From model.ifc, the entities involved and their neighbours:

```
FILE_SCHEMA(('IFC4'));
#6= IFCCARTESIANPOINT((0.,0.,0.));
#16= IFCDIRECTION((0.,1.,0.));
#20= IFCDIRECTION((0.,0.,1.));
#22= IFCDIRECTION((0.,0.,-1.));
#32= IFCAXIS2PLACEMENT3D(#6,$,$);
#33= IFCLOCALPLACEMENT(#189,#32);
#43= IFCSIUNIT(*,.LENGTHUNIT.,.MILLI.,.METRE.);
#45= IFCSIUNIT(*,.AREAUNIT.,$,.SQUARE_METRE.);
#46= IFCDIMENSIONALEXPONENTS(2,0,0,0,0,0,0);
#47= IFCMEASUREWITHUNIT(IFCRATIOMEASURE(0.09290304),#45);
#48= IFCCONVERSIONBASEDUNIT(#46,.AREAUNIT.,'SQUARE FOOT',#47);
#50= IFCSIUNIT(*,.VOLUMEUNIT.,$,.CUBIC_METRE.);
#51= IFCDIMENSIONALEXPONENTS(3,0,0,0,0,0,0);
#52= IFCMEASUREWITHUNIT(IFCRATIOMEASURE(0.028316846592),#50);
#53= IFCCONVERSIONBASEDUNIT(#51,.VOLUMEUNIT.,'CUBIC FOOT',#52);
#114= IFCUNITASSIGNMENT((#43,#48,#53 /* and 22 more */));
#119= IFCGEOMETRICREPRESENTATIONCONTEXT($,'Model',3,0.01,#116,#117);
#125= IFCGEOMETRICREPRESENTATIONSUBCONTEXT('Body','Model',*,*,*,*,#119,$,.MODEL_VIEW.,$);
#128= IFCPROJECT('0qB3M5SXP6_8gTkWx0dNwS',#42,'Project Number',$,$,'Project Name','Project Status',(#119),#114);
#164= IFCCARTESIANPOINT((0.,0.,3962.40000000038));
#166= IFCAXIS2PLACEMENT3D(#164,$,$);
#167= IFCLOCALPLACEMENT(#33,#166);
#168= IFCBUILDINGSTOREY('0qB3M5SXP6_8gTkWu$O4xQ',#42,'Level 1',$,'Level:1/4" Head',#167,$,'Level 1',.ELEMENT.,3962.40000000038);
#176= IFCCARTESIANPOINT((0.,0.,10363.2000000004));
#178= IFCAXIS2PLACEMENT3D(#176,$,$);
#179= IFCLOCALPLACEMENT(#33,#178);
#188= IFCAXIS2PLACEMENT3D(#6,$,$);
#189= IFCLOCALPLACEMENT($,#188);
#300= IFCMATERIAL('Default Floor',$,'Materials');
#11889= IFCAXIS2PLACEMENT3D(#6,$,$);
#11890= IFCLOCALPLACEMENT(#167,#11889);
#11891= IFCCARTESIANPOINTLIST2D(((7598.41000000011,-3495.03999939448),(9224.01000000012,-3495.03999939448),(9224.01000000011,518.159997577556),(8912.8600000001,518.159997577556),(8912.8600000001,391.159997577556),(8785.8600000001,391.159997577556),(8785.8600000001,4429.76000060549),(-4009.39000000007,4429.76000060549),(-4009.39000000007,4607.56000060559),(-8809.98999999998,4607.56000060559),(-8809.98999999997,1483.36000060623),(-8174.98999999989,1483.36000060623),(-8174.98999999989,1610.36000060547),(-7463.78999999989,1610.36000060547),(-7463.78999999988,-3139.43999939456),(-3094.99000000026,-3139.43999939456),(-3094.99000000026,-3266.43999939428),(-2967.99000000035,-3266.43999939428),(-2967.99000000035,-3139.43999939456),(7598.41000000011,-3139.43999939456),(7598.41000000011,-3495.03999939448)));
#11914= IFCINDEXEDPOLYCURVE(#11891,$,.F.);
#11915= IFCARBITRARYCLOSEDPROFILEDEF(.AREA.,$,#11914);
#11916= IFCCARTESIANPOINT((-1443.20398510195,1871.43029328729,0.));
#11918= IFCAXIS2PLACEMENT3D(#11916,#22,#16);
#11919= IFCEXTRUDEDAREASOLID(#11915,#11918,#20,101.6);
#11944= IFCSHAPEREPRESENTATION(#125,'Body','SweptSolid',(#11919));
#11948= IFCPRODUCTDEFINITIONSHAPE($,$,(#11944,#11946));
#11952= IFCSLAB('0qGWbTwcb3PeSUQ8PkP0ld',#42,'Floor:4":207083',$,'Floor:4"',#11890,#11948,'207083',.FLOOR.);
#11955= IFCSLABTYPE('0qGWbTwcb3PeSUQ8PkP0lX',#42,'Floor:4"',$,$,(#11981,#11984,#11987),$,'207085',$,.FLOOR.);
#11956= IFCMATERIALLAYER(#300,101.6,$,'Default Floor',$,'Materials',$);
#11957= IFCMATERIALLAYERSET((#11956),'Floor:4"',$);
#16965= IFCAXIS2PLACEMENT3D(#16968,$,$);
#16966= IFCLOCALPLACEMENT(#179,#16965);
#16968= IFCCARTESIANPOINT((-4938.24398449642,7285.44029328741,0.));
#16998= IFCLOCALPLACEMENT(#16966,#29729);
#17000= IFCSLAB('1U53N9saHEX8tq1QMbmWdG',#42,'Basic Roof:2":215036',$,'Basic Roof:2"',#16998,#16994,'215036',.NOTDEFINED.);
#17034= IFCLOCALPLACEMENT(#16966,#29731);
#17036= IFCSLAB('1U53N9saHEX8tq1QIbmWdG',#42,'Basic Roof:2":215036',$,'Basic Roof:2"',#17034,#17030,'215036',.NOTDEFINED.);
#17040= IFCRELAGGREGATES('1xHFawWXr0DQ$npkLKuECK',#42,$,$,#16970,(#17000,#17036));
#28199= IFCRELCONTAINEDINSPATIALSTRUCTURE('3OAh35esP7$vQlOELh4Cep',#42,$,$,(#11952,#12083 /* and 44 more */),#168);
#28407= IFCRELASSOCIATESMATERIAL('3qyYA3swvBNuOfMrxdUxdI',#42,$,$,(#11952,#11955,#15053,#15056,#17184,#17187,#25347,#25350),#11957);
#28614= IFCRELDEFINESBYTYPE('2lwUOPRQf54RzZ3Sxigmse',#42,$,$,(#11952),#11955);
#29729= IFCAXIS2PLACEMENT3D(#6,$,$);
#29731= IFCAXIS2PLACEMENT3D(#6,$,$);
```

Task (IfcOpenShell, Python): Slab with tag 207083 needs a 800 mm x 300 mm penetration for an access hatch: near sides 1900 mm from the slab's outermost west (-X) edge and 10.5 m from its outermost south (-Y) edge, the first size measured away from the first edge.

```python
import numpy as np
import ifcopenshell
import ifcopenshell.api.feature
import ifcopenshell.api.geometry
import ifcopenshell.api.root
import ifcopenshell.geom
import ifcopenshell.util.placement
import ifcopenshell.util.representation
import ifcopenshell.util.shape
import ifcopenshell.util.unit

model = ifcopenshell.open("model.ifc")
unit_scale = ifcopenshell.util.unit.calculate_unit_scale(model)
settings = ifcopenshell.geom.settings()


def volume(element):
    """Net volume in cubic metres, openings subtracted."""
    shape = ifcopenshell.geom.create_shape(settings, element)
    return ifcopenshell.util.shape.get_volume(shape.geometry)


slab = model.by_guid("0qGWbTwcb3PeSUQ8PkP0ld")
before = volume(slab)

# Extent in the slab's own axes, in metres. The edges named are its -X and -Y sides.
slab_shape = ifcopenshell.geom.create_shape(settings, slab)
vertices = ifcopenshell.util.shape.get_vertices(slab_shape.geometry)
x_min, y_min, bottom = vertices.min(axis=0)
top = vertices[:, 2].max()

opening = ifcopenshell.api.root.create_entity(model, ifc_class="IfcOpeningElement", name="Access hatch opening", predefined_type="OPENING")
context = ifcopenshell.util.representation.get_context(model, "Model", "Body", "MODEL_VIEW")
width, depth = 0.8, 0.3
outline = [(0.0, 0.0), (width, 0.0), (width, depth), (0.0, depth), (0.0, 0.0)]
# Overshoot both faces by 50 mm so the cut is clean.
shape = ifcopenshell.api.geometry.add_slab_representation(
    model, context=context, depth=top - bottom + 0.1, polyline=outline
)
ifcopenshell.api.geometry.assign_representation(model, product=opening, representation=shape)

matrix = ifcopenshell.util.placement.get_local_placement(slab.ObjectPlacement)
matrix[:, 3] = matrix @ np.append(np.array([x_min + 1.9, y_min + 10.5, bottom - 0.05]) / unit_scale, 1.0)
ifcopenshell.api.geometry.edit_object_placement(model, product=opening, matrix=matrix, is_si=False)
ifcopenshell.api.feature.add_feature(model, feature=opening, element=slab)

after = volume(slab)

print(f"slab volume {before:.3f} -> {after:.3f} m3")

model.write("model-out.ifc")
```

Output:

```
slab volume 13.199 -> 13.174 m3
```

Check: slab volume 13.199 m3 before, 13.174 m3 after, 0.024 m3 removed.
